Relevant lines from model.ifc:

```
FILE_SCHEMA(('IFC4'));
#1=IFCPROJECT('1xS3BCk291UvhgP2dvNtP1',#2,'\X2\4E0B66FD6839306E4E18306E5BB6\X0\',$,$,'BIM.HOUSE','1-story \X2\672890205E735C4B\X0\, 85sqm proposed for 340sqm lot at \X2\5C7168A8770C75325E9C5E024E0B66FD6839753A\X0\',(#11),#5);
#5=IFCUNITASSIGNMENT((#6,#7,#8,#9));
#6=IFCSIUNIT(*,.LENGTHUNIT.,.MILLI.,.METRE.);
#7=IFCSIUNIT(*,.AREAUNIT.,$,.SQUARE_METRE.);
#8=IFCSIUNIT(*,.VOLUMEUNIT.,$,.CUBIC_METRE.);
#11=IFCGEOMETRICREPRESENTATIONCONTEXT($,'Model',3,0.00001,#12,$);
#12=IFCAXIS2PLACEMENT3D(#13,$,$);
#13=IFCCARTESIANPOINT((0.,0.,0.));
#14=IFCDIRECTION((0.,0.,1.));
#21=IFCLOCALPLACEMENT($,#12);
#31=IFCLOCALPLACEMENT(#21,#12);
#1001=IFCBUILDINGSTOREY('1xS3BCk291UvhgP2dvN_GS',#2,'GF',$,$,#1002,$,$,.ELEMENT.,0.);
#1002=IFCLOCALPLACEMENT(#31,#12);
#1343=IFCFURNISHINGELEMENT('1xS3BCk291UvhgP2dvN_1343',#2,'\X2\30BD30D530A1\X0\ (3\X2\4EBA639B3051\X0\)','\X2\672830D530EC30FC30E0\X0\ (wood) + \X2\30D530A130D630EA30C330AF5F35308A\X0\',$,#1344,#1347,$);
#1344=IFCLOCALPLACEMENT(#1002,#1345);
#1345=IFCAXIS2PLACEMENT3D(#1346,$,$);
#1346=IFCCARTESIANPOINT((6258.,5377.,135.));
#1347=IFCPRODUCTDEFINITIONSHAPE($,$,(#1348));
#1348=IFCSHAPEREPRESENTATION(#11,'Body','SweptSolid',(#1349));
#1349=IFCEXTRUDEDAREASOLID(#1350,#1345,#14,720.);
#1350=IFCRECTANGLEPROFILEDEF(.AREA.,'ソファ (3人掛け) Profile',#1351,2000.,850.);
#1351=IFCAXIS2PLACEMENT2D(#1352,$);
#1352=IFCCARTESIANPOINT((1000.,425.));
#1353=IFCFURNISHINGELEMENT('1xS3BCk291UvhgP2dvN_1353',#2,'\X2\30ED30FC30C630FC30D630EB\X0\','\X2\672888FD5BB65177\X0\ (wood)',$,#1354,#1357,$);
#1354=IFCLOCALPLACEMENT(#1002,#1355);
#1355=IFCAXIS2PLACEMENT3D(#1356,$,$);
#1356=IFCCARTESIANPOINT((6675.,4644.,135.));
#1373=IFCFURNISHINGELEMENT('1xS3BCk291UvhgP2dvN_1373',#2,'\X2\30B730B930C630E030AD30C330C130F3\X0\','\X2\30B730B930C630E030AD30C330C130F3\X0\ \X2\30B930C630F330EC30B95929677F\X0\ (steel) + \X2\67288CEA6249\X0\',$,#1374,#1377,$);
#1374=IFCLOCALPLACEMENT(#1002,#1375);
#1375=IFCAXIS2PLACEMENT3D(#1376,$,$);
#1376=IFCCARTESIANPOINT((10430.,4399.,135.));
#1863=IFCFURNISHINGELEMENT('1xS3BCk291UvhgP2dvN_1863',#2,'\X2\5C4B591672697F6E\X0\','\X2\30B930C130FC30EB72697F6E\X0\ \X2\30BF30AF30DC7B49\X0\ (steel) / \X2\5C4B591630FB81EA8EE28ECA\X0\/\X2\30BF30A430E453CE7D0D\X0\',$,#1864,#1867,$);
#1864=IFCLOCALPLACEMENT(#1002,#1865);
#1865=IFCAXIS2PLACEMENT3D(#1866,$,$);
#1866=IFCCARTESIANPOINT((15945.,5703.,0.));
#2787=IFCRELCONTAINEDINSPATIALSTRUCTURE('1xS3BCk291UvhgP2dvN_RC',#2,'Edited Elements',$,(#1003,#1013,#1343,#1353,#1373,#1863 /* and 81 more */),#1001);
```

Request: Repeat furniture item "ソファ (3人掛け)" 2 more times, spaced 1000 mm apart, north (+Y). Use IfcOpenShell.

```python
import numpy as np
import ifcopenshell
import ifcopenshell.api.geometry
import ifcopenshell.api.root
import ifcopenshell.util.element
import ifcopenshell.util.placement
import ifcopenshell.util.unit

model = ifcopenshell.open("model.ifc")
unit_scale = ifcopenshell.util.unit.calculate_unit_scale(model)


def reuse_history(source, copy):
    """copy_class also copies each property set's owner history, people and application; keep the originals."""
    for rel in copy.IsDefinedBy:
        if rel.is_a("IfcRelDefinesByProperties") and (history := rel.RelatingPropertyDefinition.OwnerHistory):
            rel.RelatingPropertyDefinition.OwnerHistory = source.OwnerHistory
            ifcopenshell.util.element.remove_deep2(model, history)


source = model.by_id(1343)
base = ifcopenshell.util.placement.get_local_placement(source.ObjectPlacement)
step = np.array([0.0, 1.0, 0.0]) * 1 / unit_scale

for i in range(1, 3):
    copy = ifcopenshell.api.root.copy_class(model, product=source)
    copy.Representation = ifcopenshell.util.element.copy_deep(
        model, source.Representation, exclude=["IfcGeometricRepresentationContext", "IfcRepresentationMap"]
    )
    reuse_history(source, copy)
    matrix = base.copy()
    matrix[:3, 3] += i * step
    print("added at", matrix[:3, 3].round(3) + 0.0)
    ifcopenshell.api.geometry.edit_object_placement(model, product=copy, matrix=matrix, is_si=False)

model.write("model_updated.ifc")
```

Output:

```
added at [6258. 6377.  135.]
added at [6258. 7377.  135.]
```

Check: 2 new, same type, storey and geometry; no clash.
